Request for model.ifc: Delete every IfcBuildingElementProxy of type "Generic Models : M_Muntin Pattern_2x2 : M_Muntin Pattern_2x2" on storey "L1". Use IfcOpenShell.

First a look at what the model holds.

```python
import ifcopenshell
import ifcopenshell.util.element

model = ifcopenshell.open("model.ifc")
print(model.schema)
storey = next(s for s in model.by_type("IfcBuildingStorey") if s.Name == "L1")
proxies = [e for e in ifcopenshell.util.element.get_decomposition(storey) if e.is_a("IfcBuildingElementProxy")]
seen = {}
for e in proxies:
    element_type = ifcopenshell.util.element.get_type(e)
    name = element_type.Name if element_type not in (None, e) else None
    seen[name] = seen.get(name, 0) + 1
for name, count in sorted(seen.items(), key=str):
    print(count, "x", name)
```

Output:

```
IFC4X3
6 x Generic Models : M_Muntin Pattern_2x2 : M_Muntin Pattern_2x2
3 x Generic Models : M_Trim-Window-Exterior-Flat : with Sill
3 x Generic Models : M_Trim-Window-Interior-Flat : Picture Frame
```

```python
import ifcopenshell
import ifcopenshell.api.root
import ifcopenshell.util.element

model = ifcopenshell.open("model.ifc")

storey = next(s for s in model.by_type("IfcBuildingStorey") if s.Name == "L1")
proxies = [e for e in ifcopenshell.util.element.get_decomposition(storey) if e.is_a("IfcBuildingElementProxy")]
targets = [e for e in proxies if (t := ifcopenshell.util.element.get_type(e)) not in (None, e) and t.Name == "Generic Models : M_Muntin Pattern_2x2 : M_Muntin Pattern_2x2"]

for e in targets:
    ifcopenshell.api.root.remove_product(model, product=e)
print(len(targets), "removed")

model.write("model_rev.ifc")
```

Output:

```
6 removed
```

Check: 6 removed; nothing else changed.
